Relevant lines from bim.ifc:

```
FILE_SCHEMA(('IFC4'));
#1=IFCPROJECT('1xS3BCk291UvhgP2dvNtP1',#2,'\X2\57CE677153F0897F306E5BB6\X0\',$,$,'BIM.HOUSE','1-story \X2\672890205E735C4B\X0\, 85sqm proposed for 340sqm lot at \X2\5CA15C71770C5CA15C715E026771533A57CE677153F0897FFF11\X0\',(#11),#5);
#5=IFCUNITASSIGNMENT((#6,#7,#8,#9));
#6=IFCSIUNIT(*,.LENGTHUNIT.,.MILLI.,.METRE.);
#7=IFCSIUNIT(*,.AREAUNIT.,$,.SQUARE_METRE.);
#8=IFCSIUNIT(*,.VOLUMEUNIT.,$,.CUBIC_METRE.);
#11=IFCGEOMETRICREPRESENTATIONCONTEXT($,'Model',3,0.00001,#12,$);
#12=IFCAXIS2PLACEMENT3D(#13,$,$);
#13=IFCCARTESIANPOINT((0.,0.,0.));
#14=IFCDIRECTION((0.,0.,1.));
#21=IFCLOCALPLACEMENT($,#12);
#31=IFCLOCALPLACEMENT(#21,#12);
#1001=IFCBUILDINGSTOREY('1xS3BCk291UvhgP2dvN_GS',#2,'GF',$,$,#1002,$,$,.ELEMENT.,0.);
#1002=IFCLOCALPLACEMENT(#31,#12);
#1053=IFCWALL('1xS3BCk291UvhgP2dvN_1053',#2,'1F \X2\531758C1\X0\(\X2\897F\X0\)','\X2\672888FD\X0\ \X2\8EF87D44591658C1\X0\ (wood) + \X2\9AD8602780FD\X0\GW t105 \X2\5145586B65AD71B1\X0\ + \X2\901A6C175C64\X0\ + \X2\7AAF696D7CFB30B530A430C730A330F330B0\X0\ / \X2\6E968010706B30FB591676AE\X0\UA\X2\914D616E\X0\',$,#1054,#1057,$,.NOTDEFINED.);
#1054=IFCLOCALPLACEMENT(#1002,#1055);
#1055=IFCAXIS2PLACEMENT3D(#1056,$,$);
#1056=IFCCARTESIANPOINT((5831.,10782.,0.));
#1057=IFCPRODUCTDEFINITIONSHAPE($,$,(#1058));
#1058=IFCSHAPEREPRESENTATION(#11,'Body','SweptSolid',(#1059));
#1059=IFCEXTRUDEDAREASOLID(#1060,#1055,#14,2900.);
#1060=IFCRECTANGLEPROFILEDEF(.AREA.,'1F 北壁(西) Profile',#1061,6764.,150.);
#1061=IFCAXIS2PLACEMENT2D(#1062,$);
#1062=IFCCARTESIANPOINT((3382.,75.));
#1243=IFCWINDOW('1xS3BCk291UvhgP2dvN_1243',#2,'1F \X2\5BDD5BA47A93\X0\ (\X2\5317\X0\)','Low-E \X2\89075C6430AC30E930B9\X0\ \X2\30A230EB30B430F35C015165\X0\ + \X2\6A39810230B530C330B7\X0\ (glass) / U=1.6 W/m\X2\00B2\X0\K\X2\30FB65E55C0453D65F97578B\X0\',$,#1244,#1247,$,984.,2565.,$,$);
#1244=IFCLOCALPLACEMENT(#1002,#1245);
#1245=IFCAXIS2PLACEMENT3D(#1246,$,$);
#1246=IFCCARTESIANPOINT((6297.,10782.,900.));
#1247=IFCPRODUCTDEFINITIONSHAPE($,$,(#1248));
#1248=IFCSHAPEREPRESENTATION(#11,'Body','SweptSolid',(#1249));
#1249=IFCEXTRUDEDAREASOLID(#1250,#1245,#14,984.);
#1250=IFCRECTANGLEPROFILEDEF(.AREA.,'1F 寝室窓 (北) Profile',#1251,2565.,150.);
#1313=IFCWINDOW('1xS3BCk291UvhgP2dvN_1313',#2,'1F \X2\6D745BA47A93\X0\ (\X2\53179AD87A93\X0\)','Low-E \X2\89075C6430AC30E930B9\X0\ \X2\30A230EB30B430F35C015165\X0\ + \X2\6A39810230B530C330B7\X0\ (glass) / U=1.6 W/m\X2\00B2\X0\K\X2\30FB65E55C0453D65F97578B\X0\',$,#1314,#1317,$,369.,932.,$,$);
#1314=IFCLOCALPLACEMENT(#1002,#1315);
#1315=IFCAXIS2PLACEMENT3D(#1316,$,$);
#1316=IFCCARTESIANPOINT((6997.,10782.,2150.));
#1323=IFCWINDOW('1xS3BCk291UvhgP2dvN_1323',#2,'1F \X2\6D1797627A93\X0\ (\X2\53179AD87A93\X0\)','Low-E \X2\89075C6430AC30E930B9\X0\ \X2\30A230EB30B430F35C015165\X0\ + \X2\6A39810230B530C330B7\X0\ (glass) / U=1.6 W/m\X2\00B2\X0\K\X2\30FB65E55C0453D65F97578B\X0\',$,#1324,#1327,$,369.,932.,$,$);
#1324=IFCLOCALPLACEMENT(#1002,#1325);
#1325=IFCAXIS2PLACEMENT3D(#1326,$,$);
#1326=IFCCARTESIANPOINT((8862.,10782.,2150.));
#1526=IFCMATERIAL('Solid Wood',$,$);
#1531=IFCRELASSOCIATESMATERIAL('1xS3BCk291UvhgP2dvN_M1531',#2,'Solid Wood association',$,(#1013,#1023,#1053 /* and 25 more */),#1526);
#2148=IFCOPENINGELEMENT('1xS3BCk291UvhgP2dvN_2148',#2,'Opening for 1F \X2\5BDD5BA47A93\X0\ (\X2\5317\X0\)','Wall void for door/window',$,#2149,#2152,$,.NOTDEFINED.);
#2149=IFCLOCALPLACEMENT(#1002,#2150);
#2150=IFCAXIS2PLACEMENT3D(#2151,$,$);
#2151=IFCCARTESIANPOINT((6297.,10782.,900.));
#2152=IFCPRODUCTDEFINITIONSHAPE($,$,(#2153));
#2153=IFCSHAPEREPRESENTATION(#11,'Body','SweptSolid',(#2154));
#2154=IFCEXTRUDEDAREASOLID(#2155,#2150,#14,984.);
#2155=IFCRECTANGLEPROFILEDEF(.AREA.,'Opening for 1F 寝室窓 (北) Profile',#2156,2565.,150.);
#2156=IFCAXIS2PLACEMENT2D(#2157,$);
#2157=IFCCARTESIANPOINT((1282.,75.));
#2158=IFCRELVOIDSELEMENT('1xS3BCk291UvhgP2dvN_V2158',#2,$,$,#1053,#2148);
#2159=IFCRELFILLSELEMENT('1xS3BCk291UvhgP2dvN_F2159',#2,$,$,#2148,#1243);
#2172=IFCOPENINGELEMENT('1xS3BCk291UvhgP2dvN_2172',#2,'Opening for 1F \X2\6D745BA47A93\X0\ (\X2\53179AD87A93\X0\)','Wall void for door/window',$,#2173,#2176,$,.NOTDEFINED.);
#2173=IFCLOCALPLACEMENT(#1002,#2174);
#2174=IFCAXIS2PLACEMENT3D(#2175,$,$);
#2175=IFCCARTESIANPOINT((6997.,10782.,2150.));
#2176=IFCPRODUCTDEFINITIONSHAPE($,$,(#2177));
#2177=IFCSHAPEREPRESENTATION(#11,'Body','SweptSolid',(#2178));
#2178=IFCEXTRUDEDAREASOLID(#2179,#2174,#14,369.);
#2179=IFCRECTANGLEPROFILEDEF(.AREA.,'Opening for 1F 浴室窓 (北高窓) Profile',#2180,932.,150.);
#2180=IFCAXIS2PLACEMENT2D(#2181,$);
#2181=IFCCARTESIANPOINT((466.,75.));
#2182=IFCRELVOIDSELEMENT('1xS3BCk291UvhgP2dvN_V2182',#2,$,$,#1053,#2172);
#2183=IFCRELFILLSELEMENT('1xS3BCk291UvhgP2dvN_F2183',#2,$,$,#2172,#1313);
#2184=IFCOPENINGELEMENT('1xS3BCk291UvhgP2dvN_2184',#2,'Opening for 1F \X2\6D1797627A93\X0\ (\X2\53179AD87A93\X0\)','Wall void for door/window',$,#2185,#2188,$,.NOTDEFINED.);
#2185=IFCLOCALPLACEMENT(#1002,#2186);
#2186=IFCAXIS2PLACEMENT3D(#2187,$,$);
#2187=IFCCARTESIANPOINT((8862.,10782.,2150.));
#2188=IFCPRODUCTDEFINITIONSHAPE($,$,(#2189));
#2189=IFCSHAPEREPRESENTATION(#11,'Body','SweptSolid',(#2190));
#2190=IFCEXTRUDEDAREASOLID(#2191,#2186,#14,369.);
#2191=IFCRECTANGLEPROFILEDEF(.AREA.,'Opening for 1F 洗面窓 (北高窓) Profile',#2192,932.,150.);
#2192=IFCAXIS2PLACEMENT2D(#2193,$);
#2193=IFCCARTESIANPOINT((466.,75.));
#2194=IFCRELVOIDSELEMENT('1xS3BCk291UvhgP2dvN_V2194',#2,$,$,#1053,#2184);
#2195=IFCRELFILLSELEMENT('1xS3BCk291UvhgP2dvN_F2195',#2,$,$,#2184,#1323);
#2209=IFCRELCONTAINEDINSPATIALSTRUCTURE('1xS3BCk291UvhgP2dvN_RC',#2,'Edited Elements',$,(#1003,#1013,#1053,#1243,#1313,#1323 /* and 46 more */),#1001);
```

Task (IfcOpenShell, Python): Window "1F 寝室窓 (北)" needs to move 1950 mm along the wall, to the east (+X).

```python
import ifcopenshell
import ifcopenshell.api.geometry
import ifcopenshell.util.placement
import ifcopenshell.util.unit

model = ifcopenshell.open("bim.ifc")
unit_scale = ifcopenshell.util.unit.calculate_unit_scale(model)

window = model.by_guid("1xS3BCk291UvhgP2dvN_1243")
opening = window.FillsVoids[0].RelatingOpeningElement
wall = opening.VoidsElements[0].RelatingBuildingElement

wall_matrix = ifcopenshell.util.placement.get_local_placement(wall.ObjectPlacement)
shift = wall_matrix[:3, 0] * 1.95 / unit_scale
before = ifcopenshell.util.placement.get_local_placement(window.ObjectPlacement)[:3, 3].copy()

# The window is not placed relative to its opening, so move both.
for product in (opening, window):
    matrix = ifcopenshell.util.placement.get_local_placement(product.ObjectPlacement)
    matrix[:3, 3] += shift
    ifcopenshell.api.geometry.edit_object_placement(model, product=product, matrix=matrix, is_si=False)

after = ifcopenshell.util.placement.get_local_placement(window.ObjectPlacement)[:3, 3]
print("window moved by", (after - before).round(3) + 0.0)

model.write("bim_v2.ifc")
```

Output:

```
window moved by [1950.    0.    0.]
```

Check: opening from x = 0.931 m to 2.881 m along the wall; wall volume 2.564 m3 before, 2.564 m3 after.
